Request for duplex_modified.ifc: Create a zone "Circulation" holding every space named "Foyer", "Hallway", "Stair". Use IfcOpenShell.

First a look at what the model holds.

```python
import ifcopenshell

model = ifcopenshell.open("duplex_modified.ifc")
print(model.schema)
seen = {}
for space in model.by_type("IfcSpace"):
    seen[space.LongName] = seen.get(space.LongName, 0) + 1
for name, count in sorted(seen.items(), key=str):
    print(count, "x", name)
print("zones:", [z.Name for z in model.by_type("IfcZone")][:20])
```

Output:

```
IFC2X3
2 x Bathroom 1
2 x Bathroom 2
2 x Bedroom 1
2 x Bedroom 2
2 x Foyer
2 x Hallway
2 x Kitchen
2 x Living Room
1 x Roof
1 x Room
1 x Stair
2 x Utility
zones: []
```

```python
import ifcopenshell
import ifcopenshell.api.group
import ifcopenshell.api.root

model = ifcopenshell.open("duplex_modified.ifc")

names = {"Foyer", "Hallway", "Stair"}
spaces = [s for s in model.by_type("IfcSpace") if s.LongName in names]

zone = ifcopenshell.api.root.create_entity(model, ifc_class="IfcZone", name="Circulation")
ifcopenshell.api.group.assign_group(model, products=spaces, group=zone)
print(len(spaces), "spaces in", zone.Name)

model.write("duplex_modified_v2.ifc")
```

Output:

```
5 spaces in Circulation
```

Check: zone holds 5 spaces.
